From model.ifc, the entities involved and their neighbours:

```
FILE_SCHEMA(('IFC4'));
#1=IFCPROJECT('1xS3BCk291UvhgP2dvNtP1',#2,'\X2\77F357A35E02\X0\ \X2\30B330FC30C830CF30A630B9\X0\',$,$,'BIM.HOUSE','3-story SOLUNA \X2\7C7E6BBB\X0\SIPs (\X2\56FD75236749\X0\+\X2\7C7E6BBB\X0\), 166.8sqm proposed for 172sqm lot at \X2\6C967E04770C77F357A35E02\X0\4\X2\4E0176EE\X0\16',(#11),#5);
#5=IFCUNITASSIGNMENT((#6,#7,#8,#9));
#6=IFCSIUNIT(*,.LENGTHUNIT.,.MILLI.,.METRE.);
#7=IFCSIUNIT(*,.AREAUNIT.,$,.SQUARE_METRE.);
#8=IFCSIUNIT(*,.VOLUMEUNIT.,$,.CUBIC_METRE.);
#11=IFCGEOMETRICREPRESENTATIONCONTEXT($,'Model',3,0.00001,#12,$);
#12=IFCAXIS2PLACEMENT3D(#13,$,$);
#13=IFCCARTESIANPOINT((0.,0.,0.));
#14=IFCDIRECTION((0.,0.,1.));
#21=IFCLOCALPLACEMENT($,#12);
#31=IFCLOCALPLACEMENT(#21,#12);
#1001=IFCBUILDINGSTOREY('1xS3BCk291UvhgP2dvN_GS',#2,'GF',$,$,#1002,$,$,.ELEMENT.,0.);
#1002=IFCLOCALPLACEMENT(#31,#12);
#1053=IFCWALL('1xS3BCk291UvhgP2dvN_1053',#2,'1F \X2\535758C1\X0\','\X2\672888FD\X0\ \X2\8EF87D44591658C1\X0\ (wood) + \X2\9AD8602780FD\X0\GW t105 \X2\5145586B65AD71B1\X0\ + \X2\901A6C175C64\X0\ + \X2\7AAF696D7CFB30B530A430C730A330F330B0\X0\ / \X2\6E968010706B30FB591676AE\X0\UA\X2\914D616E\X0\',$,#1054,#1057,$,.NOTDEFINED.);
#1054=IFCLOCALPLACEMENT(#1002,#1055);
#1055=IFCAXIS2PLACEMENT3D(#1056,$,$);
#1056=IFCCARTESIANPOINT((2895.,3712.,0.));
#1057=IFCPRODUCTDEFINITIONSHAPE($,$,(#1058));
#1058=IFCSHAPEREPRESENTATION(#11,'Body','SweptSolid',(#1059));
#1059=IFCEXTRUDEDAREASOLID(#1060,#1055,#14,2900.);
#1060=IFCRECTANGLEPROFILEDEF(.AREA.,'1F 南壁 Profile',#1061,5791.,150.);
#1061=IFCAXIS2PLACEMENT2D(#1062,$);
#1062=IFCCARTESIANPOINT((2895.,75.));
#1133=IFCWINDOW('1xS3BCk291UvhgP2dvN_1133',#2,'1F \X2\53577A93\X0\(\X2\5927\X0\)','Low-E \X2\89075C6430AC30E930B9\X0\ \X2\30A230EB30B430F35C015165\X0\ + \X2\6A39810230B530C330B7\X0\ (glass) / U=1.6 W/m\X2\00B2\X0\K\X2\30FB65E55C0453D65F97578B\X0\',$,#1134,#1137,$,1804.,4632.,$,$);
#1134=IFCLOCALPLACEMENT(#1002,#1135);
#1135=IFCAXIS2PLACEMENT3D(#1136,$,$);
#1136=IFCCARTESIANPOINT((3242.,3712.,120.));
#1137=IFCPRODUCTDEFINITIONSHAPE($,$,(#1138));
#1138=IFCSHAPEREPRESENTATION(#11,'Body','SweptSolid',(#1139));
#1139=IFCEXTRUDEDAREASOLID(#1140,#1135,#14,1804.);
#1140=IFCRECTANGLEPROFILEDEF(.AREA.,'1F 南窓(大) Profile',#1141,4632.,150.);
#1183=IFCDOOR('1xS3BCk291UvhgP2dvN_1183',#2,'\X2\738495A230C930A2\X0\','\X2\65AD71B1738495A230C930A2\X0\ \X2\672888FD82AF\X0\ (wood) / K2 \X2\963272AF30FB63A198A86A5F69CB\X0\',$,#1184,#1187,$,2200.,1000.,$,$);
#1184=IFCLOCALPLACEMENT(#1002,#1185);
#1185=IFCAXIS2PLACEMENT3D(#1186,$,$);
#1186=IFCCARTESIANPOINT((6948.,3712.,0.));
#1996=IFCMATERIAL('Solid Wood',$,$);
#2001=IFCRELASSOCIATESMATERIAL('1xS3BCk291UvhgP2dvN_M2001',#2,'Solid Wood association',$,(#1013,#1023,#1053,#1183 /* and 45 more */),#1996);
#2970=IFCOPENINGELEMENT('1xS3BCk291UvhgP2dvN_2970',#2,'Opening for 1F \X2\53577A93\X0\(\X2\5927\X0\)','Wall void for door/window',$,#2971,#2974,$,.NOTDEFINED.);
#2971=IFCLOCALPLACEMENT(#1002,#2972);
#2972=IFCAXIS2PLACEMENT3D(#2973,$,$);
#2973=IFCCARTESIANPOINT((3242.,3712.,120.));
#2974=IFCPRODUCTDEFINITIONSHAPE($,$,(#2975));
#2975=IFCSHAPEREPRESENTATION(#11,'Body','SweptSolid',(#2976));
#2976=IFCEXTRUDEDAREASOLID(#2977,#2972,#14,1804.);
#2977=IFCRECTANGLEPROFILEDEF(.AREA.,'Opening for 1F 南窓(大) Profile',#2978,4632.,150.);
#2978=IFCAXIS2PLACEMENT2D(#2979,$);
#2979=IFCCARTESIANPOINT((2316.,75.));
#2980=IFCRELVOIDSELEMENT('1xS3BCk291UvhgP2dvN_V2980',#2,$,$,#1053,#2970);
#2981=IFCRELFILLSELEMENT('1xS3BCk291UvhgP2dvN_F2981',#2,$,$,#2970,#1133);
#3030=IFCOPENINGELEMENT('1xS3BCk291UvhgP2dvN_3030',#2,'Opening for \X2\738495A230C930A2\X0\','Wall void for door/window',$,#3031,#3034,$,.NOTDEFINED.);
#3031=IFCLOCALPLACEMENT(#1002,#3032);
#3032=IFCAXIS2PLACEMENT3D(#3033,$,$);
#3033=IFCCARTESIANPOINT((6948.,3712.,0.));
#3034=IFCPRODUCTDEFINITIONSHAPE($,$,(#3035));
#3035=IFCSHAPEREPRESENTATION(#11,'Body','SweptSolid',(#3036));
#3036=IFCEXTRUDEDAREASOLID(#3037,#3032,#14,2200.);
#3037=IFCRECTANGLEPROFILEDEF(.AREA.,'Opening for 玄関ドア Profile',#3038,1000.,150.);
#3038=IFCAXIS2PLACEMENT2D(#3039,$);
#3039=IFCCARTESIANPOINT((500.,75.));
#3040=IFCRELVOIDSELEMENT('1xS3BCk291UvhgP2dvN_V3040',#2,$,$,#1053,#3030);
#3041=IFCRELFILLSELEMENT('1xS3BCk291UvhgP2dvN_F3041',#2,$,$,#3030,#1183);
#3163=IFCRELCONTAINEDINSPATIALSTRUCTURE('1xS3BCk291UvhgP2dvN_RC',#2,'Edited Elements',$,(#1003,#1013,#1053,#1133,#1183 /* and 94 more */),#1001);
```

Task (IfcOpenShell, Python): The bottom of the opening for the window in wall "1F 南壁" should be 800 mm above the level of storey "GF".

```python
import numpy as np
import ifcopenshell
import ifcopenshell.api.geometry
import ifcopenshell.geom
import ifcopenshell.util.element
import ifcopenshell.util.placement
import ifcopenshell.util.shape
import ifcopenshell.util.unit

model = ifcopenshell.open("model.ifc")
unit_scale = ifcopenshell.util.unit.calculate_unit_scale(model)

window = model.by_guid("1xS3BCk291UvhgP2dvN_1133")
opening = window.FillsVoids[0].RelatingOpeningElement
storey = ifcopenshell.util.element.get_container(window, ifc_class="IfcBuildingStorey")
level = ifcopenshell.util.placement.get_local_placement(storey.ObjectPlacement)[2, 3]

# The opening's origin need not be at the sill, so measure its lowest point.
shape = ifcopenshell.geom.create_shape(ifcopenshell.geom.settings(), opening)
bottom = ifcopenshell.util.shape.get_shape_bottom_elevation(shape, shape.geometry) / unit_scale
dz = level + 0.8 / unit_scale - bottom

shift = np.array([0.0, 0.0, dz])
# The window is not placed relative to its opening, so move both.
for product in (opening, window):
    matrix = ifcopenshell.util.placement.get_local_placement(product.ObjectPlacement)
    matrix[:3, 3] += shift
    ifcopenshell.api.geometry.edit_object_placement(model, product=product, matrix=matrix, is_si=False)

print(f"moved by {dz * unit_scale:+.3f} m")

model.write("model_updated.ifc")
```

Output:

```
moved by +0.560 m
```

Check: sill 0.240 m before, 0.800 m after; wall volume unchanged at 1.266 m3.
